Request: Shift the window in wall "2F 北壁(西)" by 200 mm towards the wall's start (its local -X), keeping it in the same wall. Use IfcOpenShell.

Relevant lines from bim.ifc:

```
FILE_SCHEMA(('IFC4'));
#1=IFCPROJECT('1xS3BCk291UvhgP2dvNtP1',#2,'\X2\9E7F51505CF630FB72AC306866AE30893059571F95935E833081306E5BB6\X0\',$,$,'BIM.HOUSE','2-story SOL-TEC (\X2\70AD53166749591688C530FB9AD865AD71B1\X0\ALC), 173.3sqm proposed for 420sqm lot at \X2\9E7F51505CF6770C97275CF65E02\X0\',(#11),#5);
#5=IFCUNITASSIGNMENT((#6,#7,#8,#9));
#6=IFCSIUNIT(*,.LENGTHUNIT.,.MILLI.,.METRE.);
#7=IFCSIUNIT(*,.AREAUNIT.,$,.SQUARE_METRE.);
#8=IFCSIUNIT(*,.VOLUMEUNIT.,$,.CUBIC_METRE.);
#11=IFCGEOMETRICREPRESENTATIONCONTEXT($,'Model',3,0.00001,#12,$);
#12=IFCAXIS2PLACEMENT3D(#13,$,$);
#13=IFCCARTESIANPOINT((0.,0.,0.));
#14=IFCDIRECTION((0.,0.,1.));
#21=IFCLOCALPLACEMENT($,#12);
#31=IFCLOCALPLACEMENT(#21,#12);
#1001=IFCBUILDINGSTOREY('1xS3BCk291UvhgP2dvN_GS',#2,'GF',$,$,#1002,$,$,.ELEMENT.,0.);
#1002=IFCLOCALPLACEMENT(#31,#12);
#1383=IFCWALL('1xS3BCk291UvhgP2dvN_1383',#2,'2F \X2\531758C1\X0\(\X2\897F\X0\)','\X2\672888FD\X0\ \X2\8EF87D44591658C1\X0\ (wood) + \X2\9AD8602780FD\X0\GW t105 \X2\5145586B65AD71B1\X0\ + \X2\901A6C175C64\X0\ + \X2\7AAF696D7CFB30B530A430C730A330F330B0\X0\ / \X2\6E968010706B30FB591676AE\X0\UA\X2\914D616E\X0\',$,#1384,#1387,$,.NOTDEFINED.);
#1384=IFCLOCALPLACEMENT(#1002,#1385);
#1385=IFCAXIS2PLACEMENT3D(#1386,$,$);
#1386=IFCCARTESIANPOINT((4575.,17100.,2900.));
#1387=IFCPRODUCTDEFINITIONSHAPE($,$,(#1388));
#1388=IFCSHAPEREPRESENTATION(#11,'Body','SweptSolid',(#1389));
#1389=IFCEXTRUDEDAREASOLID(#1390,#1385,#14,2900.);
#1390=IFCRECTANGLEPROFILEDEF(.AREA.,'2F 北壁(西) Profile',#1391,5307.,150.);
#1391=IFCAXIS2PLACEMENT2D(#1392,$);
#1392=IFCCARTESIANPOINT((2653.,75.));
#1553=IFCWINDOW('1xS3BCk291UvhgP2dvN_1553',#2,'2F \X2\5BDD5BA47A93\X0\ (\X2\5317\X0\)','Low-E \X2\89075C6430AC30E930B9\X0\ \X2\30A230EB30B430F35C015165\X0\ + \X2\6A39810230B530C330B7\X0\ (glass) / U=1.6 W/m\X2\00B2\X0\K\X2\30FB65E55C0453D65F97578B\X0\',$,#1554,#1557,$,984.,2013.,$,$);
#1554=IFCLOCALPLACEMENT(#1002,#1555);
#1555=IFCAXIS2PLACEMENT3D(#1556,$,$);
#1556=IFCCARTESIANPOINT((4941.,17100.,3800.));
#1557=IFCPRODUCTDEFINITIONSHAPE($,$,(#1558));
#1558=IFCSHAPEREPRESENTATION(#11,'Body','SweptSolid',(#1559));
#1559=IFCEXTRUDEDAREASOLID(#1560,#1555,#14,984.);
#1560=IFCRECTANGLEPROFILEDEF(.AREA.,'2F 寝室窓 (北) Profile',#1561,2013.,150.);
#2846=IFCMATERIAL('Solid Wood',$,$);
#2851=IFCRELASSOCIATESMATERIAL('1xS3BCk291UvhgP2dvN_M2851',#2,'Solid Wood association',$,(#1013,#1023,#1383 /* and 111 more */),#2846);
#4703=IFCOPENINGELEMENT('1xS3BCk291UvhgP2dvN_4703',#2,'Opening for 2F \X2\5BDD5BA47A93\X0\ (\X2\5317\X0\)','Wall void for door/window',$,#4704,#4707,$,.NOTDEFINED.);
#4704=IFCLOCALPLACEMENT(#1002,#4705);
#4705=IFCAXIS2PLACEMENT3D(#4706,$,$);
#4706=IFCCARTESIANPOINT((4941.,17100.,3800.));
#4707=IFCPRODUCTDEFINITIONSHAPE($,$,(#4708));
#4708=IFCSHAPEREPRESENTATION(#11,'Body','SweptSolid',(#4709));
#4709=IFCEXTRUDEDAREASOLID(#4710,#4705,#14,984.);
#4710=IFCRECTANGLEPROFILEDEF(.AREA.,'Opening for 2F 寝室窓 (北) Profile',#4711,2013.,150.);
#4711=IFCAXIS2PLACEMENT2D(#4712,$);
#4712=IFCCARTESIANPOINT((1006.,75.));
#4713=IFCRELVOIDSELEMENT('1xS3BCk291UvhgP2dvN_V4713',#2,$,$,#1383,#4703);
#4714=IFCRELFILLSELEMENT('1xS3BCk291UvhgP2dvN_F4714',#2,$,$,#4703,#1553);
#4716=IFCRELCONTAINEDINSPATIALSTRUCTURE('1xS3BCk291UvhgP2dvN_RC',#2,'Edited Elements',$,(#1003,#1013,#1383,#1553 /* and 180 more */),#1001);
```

```python
import ifcopenshell
import ifcopenshell.api.geometry
import ifcopenshell.util.placement
import ifcopenshell.util.unit

model = ifcopenshell.open("bim.ifc")
unit_scale = ifcopenshell.util.unit.calculate_unit_scale(model)

window = model.by_guid("1xS3BCk291UvhgP2dvN_1553")
opening = window.FillsVoids[0].RelatingOpeningElement
wall = opening.VoidsElements[0].RelatingBuildingElement

wall_matrix = ifcopenshell.util.placement.get_local_placement(wall.ObjectPlacement)
shift = wall_matrix[:3, 0] * -0.2 / unit_scale
before = ifcopenshell.util.placement.get_local_placement(window.ObjectPlacement)[:3, 3].copy()

# The window is not placed relative to its opening, so move both.
for product in (opening, window):
    matrix = ifcopenshell.util.placement.get_local_placement(product.ObjectPlacement)
    matrix[:3, 3] += shift
    ifcopenshell.api.geometry.edit_object_placement(model, product=product, matrix=matrix, is_si=False)

after = ifcopenshell.util.placement.get_local_placement(window.ObjectPlacement)[:3, 3]
print("window moved by", (after - before).round(3) + 0.0)

model.write("bim_v2.ifc")
```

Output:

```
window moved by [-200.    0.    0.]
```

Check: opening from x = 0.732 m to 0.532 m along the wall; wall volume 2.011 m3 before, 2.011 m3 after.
